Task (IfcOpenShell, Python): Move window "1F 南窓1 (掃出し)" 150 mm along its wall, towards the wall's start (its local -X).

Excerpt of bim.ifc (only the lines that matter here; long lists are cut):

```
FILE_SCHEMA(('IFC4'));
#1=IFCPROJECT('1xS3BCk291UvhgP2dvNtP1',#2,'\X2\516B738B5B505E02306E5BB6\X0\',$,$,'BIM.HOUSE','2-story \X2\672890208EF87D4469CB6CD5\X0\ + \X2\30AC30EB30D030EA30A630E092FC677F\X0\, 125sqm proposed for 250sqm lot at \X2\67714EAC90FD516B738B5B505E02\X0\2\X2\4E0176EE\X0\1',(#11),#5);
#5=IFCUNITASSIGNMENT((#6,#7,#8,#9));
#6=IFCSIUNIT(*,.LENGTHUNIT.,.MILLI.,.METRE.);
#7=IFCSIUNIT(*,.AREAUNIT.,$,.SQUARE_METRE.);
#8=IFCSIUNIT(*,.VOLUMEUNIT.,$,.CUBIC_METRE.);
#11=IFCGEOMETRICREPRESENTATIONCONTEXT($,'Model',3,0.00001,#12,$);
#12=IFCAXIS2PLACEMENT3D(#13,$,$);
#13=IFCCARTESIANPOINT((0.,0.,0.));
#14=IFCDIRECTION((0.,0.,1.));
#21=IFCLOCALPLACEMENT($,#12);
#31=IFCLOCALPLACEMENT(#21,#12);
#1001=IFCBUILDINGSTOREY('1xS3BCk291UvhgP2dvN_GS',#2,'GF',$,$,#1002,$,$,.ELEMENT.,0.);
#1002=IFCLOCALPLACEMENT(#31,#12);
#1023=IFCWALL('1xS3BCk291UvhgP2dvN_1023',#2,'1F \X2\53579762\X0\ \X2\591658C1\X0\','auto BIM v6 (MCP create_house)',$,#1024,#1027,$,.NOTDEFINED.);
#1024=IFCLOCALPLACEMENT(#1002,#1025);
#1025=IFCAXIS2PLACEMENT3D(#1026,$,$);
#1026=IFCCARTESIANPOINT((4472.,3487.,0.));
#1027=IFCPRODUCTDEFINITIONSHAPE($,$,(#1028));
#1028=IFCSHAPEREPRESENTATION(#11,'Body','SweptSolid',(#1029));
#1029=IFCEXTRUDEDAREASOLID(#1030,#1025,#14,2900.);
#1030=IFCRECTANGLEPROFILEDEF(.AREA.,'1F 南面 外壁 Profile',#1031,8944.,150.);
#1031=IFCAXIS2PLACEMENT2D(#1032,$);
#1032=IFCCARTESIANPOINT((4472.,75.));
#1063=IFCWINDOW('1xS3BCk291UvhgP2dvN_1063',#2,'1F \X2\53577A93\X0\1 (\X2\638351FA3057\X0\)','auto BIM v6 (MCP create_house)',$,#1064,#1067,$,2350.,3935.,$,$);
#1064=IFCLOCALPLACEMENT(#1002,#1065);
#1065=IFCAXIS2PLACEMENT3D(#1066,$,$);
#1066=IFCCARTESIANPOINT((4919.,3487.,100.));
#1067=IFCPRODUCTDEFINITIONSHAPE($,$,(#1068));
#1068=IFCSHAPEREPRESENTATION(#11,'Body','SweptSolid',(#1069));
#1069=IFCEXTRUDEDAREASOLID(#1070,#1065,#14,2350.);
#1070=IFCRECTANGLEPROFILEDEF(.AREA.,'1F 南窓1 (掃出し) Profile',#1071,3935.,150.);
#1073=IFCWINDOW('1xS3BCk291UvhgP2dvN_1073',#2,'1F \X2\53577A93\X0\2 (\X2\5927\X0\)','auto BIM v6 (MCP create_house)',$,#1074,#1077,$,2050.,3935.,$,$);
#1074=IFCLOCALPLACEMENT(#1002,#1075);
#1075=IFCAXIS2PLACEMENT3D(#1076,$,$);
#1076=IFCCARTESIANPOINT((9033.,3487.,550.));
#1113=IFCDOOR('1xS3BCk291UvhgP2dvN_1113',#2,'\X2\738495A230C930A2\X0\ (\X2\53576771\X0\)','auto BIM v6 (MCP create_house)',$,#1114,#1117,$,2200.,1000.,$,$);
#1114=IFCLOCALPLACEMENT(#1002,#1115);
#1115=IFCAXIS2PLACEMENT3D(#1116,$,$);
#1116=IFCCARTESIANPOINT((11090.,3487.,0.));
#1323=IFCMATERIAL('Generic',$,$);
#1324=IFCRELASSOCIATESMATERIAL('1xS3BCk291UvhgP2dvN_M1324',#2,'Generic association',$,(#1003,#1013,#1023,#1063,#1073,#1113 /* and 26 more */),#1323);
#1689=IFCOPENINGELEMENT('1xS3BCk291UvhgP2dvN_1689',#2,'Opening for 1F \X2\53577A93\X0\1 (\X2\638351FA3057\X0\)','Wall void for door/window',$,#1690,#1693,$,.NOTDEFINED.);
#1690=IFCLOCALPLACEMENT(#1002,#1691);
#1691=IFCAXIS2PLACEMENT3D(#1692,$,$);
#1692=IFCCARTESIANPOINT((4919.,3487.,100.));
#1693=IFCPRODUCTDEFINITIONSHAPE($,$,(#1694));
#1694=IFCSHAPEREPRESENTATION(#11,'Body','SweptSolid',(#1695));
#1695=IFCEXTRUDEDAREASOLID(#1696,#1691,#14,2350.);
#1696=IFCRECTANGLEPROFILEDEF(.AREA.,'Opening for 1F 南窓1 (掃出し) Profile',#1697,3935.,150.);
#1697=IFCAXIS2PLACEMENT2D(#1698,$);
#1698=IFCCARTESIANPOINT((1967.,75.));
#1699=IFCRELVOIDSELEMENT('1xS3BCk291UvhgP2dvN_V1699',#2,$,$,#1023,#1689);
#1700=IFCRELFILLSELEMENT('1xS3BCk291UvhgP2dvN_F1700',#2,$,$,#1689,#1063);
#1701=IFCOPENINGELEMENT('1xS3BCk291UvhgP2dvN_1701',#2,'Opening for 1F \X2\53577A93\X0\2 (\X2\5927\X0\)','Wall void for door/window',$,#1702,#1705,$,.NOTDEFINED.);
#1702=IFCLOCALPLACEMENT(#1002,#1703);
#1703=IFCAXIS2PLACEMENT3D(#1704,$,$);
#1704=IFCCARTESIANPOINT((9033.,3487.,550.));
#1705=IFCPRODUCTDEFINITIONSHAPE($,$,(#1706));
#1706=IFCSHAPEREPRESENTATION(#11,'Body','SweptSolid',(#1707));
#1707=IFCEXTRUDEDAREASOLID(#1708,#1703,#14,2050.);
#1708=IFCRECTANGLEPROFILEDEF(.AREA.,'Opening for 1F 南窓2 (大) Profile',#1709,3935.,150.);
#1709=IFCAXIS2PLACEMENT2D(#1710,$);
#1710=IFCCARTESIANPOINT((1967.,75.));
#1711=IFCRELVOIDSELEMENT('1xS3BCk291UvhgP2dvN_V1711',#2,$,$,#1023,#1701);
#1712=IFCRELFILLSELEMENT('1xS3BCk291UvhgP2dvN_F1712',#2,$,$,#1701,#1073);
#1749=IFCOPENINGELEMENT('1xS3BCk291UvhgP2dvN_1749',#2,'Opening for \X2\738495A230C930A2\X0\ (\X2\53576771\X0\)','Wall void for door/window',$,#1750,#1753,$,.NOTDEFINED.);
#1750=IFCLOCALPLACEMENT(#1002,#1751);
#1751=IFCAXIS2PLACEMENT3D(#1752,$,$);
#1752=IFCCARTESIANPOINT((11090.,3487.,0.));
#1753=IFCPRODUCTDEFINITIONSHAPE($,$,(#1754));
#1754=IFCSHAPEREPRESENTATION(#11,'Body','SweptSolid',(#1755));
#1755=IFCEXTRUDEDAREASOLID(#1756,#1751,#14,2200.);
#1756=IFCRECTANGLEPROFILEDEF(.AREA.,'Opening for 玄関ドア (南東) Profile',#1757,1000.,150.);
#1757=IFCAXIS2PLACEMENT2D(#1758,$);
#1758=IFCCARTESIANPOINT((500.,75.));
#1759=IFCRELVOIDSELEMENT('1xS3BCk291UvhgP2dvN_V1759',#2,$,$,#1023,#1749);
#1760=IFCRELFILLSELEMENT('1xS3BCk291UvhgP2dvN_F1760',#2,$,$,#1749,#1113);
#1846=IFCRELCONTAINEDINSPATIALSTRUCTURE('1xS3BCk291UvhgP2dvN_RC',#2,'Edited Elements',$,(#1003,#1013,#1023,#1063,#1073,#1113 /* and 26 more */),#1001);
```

```python
import ifcopenshell
import ifcopenshell.api.geometry
import ifcopenshell.util.placement

model = ifcopenshell.open("bim.ifc")

window = model.by_guid("1xS3BCk291UvhgP2dvN_1063")
opening = window.FillsVoids[0].RelatingOpeningElement
wall = opening.VoidsElements[0].RelatingBuildingElement

wall_matrix = ifcopenshell.util.placement.get_local_placement(wall.ObjectPlacement)
shift = wall_matrix[:3, 0] * -150.0
before = ifcopenshell.util.placement.get_local_placement(window.ObjectPlacement)[:3, 3].copy()

# The window is not placed relative to its opening, so move both.
for product in (opening, window):
    matrix = ifcopenshell.util.placement.get_local_placement(product.ObjectPlacement)
    matrix[:3, 3] += shift
    ifcopenshell.api.geometry.edit_object_placement(model, product=product, matrix=matrix, is_si=False)

after = ifcopenshell.util.placement.get_local_placement(window.ObjectPlacement)[:3, 3]
print("window moved by", (after - before).round(3) + 0.0)

model.write("bim_edited.ifc")
```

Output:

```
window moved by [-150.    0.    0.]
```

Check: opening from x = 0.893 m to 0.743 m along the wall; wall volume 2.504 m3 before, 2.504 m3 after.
